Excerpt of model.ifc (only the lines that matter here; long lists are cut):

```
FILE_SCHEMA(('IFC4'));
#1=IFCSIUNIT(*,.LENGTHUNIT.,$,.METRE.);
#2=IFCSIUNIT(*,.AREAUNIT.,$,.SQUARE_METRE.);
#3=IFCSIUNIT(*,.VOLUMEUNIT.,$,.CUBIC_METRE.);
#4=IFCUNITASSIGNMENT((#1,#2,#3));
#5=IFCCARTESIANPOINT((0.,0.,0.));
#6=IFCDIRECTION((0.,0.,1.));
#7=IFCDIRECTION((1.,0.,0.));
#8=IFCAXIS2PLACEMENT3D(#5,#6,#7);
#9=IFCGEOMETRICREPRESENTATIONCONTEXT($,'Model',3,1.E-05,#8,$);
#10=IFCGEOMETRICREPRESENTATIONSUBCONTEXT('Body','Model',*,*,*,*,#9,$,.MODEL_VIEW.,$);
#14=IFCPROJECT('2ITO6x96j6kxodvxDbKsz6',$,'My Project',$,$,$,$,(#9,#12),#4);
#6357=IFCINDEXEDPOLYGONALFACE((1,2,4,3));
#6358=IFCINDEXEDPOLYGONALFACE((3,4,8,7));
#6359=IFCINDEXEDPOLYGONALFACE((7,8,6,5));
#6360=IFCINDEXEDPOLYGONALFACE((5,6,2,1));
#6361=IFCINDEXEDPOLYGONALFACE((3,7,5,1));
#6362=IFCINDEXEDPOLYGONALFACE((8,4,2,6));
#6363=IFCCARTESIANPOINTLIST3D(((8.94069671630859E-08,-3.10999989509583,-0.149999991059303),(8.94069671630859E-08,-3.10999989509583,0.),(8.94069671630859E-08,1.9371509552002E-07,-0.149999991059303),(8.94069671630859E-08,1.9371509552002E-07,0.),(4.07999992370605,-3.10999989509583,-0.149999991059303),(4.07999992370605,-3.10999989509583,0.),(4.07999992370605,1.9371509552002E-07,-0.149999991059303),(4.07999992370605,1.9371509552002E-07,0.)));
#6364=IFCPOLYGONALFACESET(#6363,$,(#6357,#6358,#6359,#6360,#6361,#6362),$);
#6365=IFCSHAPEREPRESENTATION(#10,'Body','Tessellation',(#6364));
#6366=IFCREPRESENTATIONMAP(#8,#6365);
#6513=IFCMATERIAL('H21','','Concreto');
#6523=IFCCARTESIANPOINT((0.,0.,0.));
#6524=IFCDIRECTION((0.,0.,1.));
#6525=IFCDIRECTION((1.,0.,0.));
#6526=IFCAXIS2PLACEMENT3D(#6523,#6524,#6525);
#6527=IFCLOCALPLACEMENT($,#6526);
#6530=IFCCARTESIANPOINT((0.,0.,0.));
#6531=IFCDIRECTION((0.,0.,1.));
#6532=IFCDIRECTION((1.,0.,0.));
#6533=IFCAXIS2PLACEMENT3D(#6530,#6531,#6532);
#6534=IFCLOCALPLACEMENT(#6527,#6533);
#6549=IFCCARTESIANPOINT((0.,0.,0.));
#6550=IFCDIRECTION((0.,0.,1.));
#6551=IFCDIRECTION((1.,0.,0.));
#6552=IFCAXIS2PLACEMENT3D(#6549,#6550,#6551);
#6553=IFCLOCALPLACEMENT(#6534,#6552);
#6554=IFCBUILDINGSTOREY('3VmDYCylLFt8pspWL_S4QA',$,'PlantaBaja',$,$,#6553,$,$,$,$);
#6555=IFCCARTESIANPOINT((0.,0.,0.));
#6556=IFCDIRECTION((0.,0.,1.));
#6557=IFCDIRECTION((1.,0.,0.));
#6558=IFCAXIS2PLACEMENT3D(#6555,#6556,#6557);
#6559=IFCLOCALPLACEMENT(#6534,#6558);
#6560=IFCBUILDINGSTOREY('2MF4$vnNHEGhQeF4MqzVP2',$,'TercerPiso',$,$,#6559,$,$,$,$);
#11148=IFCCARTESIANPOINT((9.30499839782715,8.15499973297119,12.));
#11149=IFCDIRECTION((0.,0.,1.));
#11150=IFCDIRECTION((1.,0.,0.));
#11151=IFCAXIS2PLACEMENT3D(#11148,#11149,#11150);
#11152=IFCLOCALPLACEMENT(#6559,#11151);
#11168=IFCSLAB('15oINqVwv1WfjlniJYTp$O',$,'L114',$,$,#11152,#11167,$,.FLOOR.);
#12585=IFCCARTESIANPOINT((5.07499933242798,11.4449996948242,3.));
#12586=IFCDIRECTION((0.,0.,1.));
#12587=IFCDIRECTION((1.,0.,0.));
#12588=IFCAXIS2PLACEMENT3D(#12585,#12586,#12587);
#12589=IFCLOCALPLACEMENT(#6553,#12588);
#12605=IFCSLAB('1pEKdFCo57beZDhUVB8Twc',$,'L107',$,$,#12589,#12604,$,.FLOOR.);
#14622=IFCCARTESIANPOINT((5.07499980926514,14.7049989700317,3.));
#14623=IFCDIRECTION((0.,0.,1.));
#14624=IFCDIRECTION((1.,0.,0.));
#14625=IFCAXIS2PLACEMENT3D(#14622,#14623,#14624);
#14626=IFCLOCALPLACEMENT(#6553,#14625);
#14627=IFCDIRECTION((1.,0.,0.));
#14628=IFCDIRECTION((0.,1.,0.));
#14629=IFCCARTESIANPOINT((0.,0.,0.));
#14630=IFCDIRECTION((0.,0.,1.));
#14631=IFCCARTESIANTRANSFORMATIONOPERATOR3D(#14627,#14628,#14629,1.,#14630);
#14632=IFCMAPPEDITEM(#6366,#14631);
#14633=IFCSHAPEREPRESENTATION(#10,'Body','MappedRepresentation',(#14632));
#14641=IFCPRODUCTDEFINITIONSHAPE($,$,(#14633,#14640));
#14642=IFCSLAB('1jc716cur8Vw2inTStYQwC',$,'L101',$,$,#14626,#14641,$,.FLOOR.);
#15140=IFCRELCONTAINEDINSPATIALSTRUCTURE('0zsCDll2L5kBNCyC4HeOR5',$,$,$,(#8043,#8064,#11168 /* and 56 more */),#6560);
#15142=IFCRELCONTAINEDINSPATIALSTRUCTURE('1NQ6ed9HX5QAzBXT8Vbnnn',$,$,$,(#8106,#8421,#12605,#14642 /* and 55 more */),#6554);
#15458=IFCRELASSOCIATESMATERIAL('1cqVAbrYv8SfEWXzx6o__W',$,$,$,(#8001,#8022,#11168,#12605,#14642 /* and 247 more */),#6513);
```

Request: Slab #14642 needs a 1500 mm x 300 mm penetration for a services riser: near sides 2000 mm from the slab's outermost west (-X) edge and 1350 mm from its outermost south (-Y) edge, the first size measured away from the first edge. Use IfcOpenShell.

```python
import numpy as np
import ifcopenshell
import ifcopenshell.api.feature
import ifcopenshell.api.geometry
import ifcopenshell.api.root
import ifcopenshell.geom
import ifcopenshell.util.placement
import ifcopenshell.util.representation
import ifcopenshell.util.shape
import ifcopenshell.util.unit

model = ifcopenshell.open("model.ifc")
unit_scale = ifcopenshell.util.unit.calculate_unit_scale(model)
settings = ifcopenshell.geom.settings()


def volume(element):
    """Net volume in cubic metres, openings subtracted."""
    shape = ifcopenshell.geom.create_shape(settings, element)
    return ifcopenshell.util.shape.get_volume(shape.geometry)


slab = model.by_guid("1jc716cur8Vw2inTStYQwC")
before = volume(slab)

# Extent in the slab's own axes, in metres. The edges named are its -X and -Y sides.
slab_shape = ifcopenshell.geom.create_shape(settings, slab)
vertices = ifcopenshell.util.shape.get_vertices(slab_shape.geometry)
x_min, y_min, bottom = vertices.min(axis=0)
top = vertices[:, 2].max()

opening = ifcopenshell.api.root.create_entity(model, ifc_class="IfcOpeningElement", name="Services riser opening", predefined_type="OPENING")
context = ifcopenshell.util.representation.get_context(model, "Model", "Body", "MODEL_VIEW")
width, depth = 1.5, 0.3
outline = [(0.0, 0.0), (width, 0.0), (width, depth), (0.0, depth), (0.0, 0.0)]
# Overshoot both faces by 50 mm so the cut is clean.
shape = ifcopenshell.api.geometry.add_slab_representation(
    model, context=context, depth=top - bottom + 0.1, polyline=outline
)
ifcopenshell.api.geometry.assign_representation(model, product=opening, representation=shape)

matrix = ifcopenshell.util.placement.get_local_placement(slab.ObjectPlacement)
matrix[:, 3] = matrix @ np.append(np.array([x_min + 2, y_min + 1.35, bottom - 0.05]) / unit_scale, 1.0)
ifcopenshell.api.geometry.edit_object_placement(model, product=opening, matrix=matrix, is_si=False)
ifcopenshell.api.feature.add_feature(model, feature=opening, element=slab)

after = volume(slab)

print(f"slab volume {before:.3f} -> {after:.3f} m3")

model.write("model-out.ifc")
```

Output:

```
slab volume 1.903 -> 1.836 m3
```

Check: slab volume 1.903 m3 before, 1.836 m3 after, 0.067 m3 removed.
